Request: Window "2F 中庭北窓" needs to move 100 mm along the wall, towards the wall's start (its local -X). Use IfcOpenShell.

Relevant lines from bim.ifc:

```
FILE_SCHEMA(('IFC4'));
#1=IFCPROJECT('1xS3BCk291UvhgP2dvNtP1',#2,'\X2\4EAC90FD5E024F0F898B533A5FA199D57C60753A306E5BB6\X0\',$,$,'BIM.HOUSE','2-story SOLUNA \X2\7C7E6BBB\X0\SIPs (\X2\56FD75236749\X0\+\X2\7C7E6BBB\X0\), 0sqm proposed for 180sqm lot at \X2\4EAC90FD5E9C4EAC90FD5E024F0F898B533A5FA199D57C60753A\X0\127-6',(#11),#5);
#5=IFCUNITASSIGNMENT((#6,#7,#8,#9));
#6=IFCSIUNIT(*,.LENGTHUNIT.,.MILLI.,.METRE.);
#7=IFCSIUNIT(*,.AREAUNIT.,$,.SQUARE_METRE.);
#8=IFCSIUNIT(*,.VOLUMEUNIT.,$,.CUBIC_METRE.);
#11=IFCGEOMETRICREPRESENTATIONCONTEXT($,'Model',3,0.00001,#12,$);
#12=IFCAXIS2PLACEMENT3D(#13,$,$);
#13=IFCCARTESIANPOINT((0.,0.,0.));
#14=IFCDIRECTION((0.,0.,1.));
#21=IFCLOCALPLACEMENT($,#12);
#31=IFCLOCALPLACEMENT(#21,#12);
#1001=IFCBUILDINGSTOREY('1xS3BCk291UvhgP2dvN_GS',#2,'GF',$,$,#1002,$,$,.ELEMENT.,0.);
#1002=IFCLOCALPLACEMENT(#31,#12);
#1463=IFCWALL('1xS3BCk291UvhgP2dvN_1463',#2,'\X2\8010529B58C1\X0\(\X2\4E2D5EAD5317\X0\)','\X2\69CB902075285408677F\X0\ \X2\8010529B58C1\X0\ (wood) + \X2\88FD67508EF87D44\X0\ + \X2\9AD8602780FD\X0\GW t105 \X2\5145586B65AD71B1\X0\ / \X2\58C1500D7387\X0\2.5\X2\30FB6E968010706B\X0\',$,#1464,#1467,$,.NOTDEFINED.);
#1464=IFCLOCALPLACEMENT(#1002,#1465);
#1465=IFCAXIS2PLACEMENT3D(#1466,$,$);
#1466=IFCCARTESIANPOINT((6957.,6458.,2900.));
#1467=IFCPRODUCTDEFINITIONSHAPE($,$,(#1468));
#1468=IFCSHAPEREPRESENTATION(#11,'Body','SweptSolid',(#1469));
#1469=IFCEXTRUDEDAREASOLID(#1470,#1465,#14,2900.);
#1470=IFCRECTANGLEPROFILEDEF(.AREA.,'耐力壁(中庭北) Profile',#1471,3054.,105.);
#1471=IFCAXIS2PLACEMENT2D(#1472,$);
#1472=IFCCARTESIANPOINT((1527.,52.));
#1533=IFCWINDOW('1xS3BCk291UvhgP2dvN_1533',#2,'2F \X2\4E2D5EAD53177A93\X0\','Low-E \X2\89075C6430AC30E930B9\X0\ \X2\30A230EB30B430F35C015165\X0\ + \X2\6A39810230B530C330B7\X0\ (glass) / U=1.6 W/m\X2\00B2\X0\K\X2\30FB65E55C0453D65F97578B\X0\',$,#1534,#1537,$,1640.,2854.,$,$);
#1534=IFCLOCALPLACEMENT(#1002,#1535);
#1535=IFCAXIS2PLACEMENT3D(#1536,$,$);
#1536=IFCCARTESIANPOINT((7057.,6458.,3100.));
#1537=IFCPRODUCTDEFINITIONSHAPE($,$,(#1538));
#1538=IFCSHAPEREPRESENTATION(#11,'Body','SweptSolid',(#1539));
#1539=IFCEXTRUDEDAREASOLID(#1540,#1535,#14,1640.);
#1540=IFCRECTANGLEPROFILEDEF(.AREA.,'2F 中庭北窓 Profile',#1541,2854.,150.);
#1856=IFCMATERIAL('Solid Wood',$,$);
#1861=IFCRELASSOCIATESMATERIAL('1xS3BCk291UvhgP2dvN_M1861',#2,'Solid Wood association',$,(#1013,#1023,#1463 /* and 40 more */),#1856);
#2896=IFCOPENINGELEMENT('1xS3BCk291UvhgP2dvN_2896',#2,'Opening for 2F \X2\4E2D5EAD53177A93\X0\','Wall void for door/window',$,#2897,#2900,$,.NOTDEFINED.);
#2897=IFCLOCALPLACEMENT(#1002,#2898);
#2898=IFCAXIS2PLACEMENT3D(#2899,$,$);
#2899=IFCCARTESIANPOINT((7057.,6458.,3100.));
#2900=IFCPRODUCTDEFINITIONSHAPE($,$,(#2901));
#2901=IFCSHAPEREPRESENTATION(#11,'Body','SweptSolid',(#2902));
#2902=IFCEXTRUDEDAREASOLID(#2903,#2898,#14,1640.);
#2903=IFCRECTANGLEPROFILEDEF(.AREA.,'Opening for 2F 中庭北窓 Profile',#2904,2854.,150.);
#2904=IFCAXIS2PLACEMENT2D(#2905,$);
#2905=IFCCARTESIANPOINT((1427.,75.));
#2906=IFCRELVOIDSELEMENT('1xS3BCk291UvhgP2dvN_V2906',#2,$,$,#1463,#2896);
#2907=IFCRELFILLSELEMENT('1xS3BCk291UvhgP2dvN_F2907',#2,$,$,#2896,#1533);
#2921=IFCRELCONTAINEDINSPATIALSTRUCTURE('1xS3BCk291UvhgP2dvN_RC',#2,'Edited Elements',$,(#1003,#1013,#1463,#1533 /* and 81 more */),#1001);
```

```python
import ifcopenshell
import ifcopenshell.api.geometry
import ifcopenshell.util.placement

model = ifcopenshell.open("bim.ifc")

window = model.by_guid("1xS3BCk291UvhgP2dvN_1533")
opening = window.FillsVoids[0].RelatingOpeningElement
wall = opening.VoidsElements[0].RelatingBuildingElement

wall_matrix = ifcopenshell.util.placement.get_local_placement(wall.ObjectPlacement)
shift = wall_matrix[:3, 0] * -100.0
before = ifcopenshell.util.placement.get_local_placement(window.ObjectPlacement)[:3, 3].copy()

# The window is not placed relative to its opening, so move both.
for product in (opening, window):
    matrix = ifcopenshell.util.placement.get_local_placement(product.ObjectPlacement)
    matrix[:3, 3] += shift
    ifcopenshell.api.geometry.edit_object_placement(model, product=product, matrix=matrix, is_si=False)

after = ifcopenshell.util.placement.get_local_placement(window.ObjectPlacement)[:3, 3]
print("window moved by", (after - before).round(3) + 0.0)

model.write("bim_v2.ifc")
```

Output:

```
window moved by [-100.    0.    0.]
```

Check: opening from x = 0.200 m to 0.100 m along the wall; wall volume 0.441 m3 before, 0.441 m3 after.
